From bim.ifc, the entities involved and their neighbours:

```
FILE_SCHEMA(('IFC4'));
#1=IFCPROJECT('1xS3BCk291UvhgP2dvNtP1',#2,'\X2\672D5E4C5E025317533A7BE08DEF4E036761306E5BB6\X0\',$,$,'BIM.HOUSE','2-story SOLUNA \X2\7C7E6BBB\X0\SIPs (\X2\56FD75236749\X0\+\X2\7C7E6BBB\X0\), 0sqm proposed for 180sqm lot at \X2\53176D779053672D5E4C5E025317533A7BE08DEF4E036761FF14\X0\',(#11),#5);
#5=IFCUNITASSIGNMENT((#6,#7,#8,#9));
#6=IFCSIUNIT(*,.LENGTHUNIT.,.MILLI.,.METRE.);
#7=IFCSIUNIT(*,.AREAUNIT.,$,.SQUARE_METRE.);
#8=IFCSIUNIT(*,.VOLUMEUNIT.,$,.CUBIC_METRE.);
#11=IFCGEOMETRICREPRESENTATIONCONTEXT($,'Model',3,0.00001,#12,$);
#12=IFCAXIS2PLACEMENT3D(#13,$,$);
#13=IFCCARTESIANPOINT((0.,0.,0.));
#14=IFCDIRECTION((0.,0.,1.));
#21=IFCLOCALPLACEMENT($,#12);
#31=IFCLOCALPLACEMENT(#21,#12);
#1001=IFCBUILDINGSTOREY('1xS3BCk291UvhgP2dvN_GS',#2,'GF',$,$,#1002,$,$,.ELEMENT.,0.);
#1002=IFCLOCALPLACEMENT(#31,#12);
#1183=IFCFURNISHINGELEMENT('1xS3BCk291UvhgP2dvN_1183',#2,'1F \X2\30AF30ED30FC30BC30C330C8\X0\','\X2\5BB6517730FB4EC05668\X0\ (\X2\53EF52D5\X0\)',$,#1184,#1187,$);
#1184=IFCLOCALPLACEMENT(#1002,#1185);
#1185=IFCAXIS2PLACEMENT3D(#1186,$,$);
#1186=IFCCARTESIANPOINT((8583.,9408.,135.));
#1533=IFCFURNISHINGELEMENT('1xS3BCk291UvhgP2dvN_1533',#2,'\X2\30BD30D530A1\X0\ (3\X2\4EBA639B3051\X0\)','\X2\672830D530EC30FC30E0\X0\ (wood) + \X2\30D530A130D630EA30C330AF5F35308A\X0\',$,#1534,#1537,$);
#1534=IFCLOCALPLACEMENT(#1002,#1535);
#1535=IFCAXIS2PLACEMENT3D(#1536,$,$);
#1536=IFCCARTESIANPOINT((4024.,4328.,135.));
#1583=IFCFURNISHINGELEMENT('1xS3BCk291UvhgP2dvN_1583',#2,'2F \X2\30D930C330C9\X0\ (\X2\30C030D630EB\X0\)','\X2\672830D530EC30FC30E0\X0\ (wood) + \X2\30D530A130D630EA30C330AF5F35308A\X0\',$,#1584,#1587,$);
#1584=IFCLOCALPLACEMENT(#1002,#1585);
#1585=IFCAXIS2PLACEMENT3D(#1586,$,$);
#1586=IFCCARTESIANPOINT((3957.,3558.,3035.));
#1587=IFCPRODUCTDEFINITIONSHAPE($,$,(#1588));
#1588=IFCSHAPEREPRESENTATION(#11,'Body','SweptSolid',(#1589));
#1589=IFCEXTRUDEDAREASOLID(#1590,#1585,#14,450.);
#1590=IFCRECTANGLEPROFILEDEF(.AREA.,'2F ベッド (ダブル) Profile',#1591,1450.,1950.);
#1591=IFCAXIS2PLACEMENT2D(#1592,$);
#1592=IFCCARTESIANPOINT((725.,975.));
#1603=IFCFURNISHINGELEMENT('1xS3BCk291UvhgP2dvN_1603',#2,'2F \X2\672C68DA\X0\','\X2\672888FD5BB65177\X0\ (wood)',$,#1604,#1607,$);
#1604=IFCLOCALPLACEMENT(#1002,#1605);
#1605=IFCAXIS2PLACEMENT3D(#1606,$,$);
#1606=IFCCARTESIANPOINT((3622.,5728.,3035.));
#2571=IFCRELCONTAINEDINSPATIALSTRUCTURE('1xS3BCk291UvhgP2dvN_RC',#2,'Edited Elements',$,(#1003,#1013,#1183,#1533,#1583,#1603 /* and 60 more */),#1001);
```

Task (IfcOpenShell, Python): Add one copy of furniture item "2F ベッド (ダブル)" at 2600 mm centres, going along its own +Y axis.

```python
import ifcopenshell
import ifcopenshell.api.geometry
import ifcopenshell.api.root
import ifcopenshell.util.element
import ifcopenshell.util.placement

model = ifcopenshell.open("bim.ifc")


def reuse_history(source, copy):
    """copy_class also copies each property set's owner history, people and application; keep the originals."""
    for rel in copy.IsDefinedBy:
        if rel.is_a("IfcRelDefinesByProperties") and (history := rel.RelatingPropertyDefinition.OwnerHistory):
            rel.RelatingPropertyDefinition.OwnerHistory = source.OwnerHistory
            ifcopenshell.util.element.remove_deep2(model, history)


source = model.by_id(1583)
base = ifcopenshell.util.placement.get_local_placement(source.ObjectPlacement)
step = base[:3, 1] * 2600.0

for i in range(1, 2):
    copy = ifcopenshell.api.root.copy_class(model, product=source)
    copy.Representation = ifcopenshell.util.element.copy_deep(
        model, source.Representation, exclude=["IfcGeometricRepresentationContext", "IfcRepresentationMap"]
    )
    reuse_history(source, copy)
    matrix = base.copy()
    matrix[:3, 3] += i * step
    print("added at", matrix[:3, 3].round(3) + 0.0)
    ifcopenshell.api.geometry.edit_object_placement(model, product=copy, matrix=matrix, is_si=False)

model.write("bim_rev.ifc")
```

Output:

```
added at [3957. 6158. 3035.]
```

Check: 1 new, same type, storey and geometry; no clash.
